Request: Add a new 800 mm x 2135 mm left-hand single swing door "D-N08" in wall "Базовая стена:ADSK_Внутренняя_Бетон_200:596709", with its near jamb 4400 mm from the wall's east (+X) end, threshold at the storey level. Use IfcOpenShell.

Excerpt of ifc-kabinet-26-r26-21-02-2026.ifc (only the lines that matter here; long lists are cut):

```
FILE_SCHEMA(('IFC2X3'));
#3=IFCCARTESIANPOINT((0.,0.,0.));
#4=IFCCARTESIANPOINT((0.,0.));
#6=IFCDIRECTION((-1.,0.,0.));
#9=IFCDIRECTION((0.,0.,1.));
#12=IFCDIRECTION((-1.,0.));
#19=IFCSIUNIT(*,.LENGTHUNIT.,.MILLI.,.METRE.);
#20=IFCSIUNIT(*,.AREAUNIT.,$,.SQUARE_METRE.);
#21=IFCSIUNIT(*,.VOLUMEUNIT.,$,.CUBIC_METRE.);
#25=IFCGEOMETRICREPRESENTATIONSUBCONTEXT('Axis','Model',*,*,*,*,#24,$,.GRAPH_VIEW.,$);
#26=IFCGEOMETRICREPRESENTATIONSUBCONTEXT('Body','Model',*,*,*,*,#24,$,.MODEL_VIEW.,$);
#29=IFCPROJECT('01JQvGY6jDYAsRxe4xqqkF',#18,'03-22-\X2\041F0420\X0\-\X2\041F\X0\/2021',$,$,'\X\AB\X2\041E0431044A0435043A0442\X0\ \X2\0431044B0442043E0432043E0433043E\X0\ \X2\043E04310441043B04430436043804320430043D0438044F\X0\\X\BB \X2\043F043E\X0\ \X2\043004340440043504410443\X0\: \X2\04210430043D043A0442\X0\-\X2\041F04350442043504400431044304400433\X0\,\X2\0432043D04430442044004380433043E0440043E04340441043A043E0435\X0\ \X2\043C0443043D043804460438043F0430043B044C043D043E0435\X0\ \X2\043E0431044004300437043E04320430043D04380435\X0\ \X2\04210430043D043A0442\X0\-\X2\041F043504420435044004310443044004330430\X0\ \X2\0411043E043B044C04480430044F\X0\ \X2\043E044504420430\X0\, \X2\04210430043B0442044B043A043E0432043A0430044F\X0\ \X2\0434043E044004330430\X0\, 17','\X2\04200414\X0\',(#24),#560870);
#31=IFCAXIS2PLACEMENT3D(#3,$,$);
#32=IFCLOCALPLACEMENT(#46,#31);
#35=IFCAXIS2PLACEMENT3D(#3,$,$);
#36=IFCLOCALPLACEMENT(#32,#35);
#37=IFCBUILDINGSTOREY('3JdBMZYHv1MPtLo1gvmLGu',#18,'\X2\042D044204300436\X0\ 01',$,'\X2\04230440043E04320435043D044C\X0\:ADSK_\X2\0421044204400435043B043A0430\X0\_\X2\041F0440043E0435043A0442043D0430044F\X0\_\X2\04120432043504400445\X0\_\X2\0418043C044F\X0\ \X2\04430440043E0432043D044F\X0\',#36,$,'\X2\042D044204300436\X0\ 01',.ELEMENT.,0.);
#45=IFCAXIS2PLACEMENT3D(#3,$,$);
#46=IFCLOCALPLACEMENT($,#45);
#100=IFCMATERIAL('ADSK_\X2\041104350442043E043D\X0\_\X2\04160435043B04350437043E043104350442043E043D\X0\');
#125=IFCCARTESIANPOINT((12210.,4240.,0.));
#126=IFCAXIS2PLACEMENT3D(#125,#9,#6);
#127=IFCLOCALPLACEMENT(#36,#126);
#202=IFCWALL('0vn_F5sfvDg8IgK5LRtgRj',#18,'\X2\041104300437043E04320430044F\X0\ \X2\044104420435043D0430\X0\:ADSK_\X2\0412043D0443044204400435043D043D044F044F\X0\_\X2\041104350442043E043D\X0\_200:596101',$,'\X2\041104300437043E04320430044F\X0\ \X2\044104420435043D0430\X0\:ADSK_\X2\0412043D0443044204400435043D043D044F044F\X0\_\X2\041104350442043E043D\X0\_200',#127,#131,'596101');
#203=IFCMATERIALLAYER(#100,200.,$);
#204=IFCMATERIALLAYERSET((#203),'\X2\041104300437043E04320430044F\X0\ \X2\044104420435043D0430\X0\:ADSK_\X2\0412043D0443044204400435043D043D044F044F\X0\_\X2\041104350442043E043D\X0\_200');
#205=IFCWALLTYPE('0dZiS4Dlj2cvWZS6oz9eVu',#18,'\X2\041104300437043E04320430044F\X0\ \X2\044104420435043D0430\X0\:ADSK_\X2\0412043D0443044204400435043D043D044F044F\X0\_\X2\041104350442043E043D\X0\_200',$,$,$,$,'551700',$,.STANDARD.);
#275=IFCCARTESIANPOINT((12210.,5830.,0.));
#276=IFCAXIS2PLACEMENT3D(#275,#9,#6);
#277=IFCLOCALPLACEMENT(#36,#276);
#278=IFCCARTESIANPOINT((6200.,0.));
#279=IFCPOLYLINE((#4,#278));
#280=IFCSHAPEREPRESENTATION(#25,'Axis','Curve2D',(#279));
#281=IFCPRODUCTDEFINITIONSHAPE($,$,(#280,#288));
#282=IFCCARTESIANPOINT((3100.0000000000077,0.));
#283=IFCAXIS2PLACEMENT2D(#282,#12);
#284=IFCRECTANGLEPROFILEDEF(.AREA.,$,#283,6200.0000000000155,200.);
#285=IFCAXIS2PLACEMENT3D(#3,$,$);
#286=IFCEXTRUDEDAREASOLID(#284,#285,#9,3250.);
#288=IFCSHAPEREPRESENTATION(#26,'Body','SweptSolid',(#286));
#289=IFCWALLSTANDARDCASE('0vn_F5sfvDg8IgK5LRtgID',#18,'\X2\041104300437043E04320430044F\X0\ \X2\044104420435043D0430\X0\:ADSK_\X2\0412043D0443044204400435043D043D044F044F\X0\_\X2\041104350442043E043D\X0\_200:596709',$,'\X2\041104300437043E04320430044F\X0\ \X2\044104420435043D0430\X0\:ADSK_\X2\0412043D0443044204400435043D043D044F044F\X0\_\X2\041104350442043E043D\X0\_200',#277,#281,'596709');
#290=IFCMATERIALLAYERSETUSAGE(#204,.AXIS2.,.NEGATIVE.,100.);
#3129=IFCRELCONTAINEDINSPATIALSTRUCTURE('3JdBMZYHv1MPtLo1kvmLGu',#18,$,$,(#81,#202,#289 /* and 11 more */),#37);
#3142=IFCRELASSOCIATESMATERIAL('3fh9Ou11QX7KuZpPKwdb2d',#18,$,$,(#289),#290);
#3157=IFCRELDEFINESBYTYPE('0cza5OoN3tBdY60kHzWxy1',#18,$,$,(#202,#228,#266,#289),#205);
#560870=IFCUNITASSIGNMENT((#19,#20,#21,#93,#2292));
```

```python
import numpy as np
import ifcopenshell
import ifcopenshell.api.feature
import ifcopenshell.api.geometry
import ifcopenshell.api.root
import ifcopenshell.api.spatial
import ifcopenshell.api.type
import ifcopenshell.geom
import ifcopenshell.util.element
import ifcopenshell.util.placement
import ifcopenshell.util.representation
import ifcopenshell.util.shape
import ifcopenshell.util.unit

model = ifcopenshell.open("ifc-kabinet-26-r26-21-02-2026.ifc")
unit_scale = ifcopenshell.util.unit.calculate_unit_scale(model)
settings = ifcopenshell.geom.settings()


def volume(element):
    """Net volume in cubic metres, openings subtracted."""
    shape = ifcopenshell.geom.create_shape(settings, element)
    return ifcopenshell.util.shape.get_volume(shape.geometry)


wall = model.by_guid("0vn_F5sfvDg8IgK5LRtgID")
storey = ifcopenshell.util.element.get_container(wall, ifc_class="IfcBuildingStorey")
context = ifcopenshell.util.representation.get_context(model, "Model", "Body", "MODEL_VIEW")
before = volume(wall)

width, height, from_end, sill = 0.8, 2.135, 4.4, 0.0  # metres

# The wall runs along its own X axis, and the end named is its -X end.
wall_shape = ifcopenshell.geom.create_shape(settings, wall)
x, y, z = ifcopenshell.util.shape.get_vertices(wall_shape.geometry).T
start = x.min() + from_end
face, thickness = float(y.min()), float(y.max() - y.min())
wall_matrix = ifcopenshell.util.placement.get_local_placement(wall.ObjectPlacement)
level = ifcopenshell.util.placement.get_local_placement(storey.ObjectPlacement)[2, 3]


def in_wall(x, y):
    """Placement at x, y metres in the wall's axes, at sill height."""
    matrix = wall_matrix.copy()
    matrix[:, 3] = wall_matrix @ np.array([x / unit_scale, y / unit_scale, 0.0, 1.0])
    matrix[2, 3] = level + sill / unit_scale
    return matrix


# Opening: a box that overshoots both wall faces by 50 mm.
opening = ifcopenshell.api.root.create_entity(model, ifc_class="IfcOpeningElement")
box = ifcopenshell.api.geometry.add_wall_representation(
    model, context=context, length=width, height=height, thickness=thickness + 0.1
)
ifcopenshell.api.geometry.assign_representation(model, product=opening, representation=box)
ifcopenshell.api.geometry.edit_object_placement(model, product=opening, matrix=in_wall(start, face - 0.05), is_si=False)
ifcopenshell.api.feature.add_feature(model, feature=opening, element=wall)

door = ifcopenshell.api.root.create_entity(model, ifc_class="IfcDoor", name="D-N08")
door.OverallWidth, door.OverallHeight = width / unit_scale, height / unit_scale
body = ifcopenshell.api.geometry.add_door_representation(
    model,
    context=context,
    overall_width=door.OverallWidth,
    overall_height=door.OverallHeight,
    operation_type="SINGLE_SWING_LEFT",
    lining_properties={"LiningDepth": thickness / unit_scale, "ThresholdDepth": thickness / unit_scale},
)
ifcopenshell.api.geometry.assign_representation(model, product=door, representation=body)
ifcopenshell.api.spatial.assign_container(model, products=[door], relating_structure=storey)
fills = ifcopenshell.api.feature.add_filling(model, opening=opening, element=door)
fills.OwnerHistory = door.OwnerHistory  # required in IFC2X3

# IFC2X3 keeps the operation on the door style.
style = ifcopenshell.api.root.create_entity(model, ifc_class="IfcDoorStyle", name="D-N08")
style.OperationType, style.ConstructionType = "SINGLE_SWING_LEFT", "NOTDEFINED"
style.ParameterTakesPrecedence = style.Sizeable = False
ifcopenshell.api.type.assign_type(model, related_objects=[door], relating_type=style)

# The lining spans the wall, so the door starts at the wall face.
ifcopenshell.api.geometry.edit_object_placement(model, product=door, matrix=in_wall(start, face), is_si=False)

after = volume(wall)

print(f"wall volume {before:.3f} -> {after:.3f} m3")

model.write("ifc-kabinet-26-r26-21-02-2026_rev.ifc")
```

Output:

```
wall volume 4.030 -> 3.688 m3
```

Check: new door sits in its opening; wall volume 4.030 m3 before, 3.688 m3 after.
